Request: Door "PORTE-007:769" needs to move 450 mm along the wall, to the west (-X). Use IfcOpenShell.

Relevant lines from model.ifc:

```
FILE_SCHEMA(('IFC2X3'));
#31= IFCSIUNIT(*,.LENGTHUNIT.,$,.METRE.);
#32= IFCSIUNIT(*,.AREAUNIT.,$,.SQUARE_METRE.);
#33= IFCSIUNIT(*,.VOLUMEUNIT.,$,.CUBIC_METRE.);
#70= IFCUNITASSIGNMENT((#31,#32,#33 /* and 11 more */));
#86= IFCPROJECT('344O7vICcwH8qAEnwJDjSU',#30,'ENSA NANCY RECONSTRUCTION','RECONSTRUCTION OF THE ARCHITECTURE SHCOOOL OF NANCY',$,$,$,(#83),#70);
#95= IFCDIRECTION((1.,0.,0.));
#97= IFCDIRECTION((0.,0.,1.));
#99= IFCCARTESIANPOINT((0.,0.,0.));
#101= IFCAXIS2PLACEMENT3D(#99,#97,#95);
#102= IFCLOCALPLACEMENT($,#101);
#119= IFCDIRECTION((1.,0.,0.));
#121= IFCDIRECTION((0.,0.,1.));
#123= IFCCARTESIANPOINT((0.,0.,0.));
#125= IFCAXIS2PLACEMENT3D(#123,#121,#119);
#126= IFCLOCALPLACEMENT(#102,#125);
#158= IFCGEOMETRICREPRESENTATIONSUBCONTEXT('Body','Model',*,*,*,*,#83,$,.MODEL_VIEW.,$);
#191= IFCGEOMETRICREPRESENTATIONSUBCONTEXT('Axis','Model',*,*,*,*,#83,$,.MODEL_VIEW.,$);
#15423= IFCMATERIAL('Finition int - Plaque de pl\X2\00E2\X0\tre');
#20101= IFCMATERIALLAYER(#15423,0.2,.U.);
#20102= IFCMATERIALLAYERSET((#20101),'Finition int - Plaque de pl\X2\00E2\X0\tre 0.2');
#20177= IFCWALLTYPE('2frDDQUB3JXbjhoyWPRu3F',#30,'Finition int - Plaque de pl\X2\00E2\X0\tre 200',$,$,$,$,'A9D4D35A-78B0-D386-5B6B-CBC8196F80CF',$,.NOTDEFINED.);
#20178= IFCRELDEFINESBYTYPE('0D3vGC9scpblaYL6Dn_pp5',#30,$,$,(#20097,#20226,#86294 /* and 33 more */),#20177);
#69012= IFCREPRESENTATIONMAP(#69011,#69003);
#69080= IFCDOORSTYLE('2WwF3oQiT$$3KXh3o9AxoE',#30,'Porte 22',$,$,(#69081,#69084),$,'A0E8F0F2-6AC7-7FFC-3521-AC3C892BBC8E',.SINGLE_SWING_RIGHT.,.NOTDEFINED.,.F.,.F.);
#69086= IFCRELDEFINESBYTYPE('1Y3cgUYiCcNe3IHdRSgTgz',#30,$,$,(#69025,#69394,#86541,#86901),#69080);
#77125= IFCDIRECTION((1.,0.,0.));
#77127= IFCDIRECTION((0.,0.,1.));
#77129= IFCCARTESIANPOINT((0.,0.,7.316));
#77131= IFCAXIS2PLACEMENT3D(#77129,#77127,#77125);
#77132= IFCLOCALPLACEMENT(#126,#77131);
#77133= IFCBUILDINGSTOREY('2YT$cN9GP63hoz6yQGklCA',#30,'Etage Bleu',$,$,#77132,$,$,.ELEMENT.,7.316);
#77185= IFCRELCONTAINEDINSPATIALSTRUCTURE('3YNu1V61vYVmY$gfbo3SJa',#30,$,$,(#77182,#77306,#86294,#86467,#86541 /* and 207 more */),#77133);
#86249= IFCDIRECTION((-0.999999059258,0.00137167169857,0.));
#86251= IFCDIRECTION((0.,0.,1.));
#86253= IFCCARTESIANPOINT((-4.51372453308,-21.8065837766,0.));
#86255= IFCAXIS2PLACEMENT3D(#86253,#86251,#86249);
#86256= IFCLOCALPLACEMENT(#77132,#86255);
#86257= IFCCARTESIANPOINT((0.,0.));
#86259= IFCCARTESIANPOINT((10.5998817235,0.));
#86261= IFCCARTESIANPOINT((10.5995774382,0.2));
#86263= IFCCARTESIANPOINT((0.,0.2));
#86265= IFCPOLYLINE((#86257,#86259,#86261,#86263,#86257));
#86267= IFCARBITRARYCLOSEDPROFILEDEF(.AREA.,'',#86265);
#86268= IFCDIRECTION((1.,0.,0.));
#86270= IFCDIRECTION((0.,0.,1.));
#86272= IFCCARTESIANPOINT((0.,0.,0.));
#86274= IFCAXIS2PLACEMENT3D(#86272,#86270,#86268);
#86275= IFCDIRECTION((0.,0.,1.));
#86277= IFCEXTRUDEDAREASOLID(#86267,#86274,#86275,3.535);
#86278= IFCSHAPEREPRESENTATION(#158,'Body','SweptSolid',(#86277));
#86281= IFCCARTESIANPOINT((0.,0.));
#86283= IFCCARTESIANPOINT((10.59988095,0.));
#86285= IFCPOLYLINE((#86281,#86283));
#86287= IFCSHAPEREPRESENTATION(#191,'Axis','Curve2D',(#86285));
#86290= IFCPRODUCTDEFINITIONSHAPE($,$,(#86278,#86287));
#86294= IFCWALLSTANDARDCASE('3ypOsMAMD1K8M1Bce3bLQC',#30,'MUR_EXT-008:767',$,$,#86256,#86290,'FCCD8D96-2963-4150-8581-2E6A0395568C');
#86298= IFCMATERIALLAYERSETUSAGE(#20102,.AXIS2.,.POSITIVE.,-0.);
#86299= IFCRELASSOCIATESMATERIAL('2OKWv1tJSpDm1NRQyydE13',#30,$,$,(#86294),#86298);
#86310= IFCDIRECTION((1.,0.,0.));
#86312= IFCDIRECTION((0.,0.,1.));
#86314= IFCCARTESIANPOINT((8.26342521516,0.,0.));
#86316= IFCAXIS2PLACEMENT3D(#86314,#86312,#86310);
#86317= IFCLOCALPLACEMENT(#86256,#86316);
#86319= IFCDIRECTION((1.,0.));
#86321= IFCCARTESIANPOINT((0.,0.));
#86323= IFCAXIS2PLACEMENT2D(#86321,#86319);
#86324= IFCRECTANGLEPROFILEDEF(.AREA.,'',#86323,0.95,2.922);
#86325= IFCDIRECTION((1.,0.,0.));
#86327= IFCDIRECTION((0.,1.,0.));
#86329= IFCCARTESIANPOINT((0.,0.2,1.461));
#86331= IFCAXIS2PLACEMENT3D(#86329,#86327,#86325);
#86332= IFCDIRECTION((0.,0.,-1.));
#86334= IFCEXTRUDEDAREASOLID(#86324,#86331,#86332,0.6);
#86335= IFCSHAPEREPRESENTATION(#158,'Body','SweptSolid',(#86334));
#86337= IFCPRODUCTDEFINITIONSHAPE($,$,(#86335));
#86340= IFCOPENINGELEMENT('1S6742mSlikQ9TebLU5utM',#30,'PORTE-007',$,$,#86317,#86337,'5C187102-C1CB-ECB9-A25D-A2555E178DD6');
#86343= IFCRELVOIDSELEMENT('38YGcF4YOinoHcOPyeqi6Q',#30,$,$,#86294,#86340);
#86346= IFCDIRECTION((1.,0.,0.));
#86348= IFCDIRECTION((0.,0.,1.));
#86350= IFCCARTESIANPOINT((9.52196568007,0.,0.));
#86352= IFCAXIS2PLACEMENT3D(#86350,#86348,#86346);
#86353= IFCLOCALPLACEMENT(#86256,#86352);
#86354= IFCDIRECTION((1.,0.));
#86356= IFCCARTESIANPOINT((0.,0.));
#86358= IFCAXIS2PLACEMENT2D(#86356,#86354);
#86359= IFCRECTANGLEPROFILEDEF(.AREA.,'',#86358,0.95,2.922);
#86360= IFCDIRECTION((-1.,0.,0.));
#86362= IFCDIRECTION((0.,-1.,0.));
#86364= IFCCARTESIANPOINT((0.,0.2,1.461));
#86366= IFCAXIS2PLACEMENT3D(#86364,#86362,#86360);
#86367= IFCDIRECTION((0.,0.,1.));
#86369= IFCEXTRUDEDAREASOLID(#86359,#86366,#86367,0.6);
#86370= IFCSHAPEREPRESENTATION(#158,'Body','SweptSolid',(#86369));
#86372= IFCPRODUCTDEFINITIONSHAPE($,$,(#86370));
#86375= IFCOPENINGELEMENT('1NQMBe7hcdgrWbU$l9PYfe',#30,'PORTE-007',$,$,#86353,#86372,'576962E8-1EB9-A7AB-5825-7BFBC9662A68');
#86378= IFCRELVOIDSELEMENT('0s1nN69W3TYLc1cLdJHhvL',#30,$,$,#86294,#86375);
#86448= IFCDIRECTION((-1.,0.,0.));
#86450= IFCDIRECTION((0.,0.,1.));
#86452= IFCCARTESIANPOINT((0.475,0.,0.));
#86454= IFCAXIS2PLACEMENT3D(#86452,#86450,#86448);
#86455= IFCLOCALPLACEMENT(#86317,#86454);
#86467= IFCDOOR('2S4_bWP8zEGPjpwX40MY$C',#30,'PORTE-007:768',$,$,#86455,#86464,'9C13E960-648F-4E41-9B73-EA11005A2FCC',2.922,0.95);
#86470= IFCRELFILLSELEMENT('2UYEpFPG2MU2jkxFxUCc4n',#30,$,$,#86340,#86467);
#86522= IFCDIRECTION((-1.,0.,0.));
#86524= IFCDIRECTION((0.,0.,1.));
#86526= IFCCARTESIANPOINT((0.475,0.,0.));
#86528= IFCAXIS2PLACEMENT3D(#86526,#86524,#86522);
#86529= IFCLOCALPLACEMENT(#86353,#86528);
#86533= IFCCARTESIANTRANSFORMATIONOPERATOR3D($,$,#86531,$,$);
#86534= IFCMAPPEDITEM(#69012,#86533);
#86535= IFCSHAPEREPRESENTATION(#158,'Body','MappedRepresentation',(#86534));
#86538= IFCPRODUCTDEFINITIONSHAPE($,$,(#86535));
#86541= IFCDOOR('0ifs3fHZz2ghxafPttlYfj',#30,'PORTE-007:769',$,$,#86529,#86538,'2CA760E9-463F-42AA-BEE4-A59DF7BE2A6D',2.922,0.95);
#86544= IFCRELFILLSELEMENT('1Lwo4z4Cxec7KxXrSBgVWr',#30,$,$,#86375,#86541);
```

```python
import ifcopenshell
import ifcopenshell.api.geometry
import ifcopenshell.util.placement
import ifcopenshell.util.unit

model = ifcopenshell.open("model.ifc")
unit_scale = ifcopenshell.util.unit.calculate_unit_scale(model)

door = model.by_guid("0ifs3fHZz2ghxafPttlYfj")
opening = door.FillsVoids[0].RelatingOpeningElement
wall = opening.VoidsElements[0].RelatingBuildingElement

wall_matrix = ifcopenshell.util.placement.get_local_placement(wall.ObjectPlacement)
shift = wall_matrix[:3, 0] * 0.45 / unit_scale
before = ifcopenshell.util.placement.get_local_placement(door.ObjectPlacement)[:3, 3].copy()

# The door is placed relative to its opening, so it follows when the opening moves.
matrix = ifcopenshell.util.placement.get_local_placement(opening.ObjectPlacement)
matrix[:3, 3] += shift
ifcopenshell.api.geometry.edit_object_placement(
    model, product=opening, matrix=matrix, is_si=False, should_transform_children=True
)

after = ifcopenshell.util.placement.get_local_placement(door.ObjectPlacement)[:3, 3]
print("door moved by", (after - before).round(3) + 0.0)

model.write("model-out.ifc")
```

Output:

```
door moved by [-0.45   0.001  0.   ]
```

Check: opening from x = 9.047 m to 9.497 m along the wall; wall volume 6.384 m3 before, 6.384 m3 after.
